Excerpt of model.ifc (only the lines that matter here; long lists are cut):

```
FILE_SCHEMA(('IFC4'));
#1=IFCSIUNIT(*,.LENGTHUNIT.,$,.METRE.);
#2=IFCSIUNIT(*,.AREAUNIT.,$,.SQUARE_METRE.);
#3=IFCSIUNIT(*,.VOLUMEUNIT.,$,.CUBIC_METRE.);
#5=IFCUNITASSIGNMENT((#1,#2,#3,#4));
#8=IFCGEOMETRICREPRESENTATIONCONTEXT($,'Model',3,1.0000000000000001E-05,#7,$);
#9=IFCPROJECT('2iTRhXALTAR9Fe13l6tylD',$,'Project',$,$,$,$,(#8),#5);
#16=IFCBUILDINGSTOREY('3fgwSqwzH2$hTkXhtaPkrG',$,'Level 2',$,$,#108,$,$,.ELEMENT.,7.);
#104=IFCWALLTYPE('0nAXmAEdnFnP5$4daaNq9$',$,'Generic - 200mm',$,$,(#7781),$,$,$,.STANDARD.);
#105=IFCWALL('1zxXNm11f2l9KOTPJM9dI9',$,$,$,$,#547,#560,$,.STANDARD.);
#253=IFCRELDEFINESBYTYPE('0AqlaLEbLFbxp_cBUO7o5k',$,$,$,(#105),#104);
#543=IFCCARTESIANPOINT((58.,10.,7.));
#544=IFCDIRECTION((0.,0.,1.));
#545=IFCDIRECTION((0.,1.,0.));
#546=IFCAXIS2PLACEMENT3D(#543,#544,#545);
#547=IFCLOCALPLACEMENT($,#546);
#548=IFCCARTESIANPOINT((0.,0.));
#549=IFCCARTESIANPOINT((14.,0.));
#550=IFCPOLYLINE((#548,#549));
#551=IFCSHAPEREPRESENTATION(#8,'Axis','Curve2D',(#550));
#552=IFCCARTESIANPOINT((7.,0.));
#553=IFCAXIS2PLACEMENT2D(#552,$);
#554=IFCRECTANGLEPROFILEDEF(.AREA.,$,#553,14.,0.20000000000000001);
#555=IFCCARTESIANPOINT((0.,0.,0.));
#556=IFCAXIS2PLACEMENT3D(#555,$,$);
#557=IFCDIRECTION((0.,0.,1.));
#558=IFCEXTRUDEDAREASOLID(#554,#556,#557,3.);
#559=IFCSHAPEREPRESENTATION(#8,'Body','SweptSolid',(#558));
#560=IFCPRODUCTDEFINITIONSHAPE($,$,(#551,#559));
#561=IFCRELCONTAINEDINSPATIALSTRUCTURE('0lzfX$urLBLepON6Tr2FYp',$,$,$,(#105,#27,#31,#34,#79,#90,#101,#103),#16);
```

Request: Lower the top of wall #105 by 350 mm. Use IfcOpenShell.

```python
import ifcopenshell
import ifcopenshell.geom
import ifcopenshell.util.shape
import ifcopenshell.util.unit

model = ifcopenshell.open("model.ifc")
unit_scale = ifcopenshell.util.unit.calculate_unit_scale(model)
settings = ifcopenshell.geom.settings()


def volume(element):
    """Net volume in cubic metres, openings subtracted."""
    shape = ifcopenshell.geom.create_shape(settings, element)
    return ifcopenshell.util.shape.get_volume(shape.geometry)


wall = model.by_guid("1zxXNm11f2l9KOTPJM9dI9")
before = volume(wall)

body = next(r for r in wall.Representation.Representations if r.RepresentationIdentifier == "Body")
solid = body.Items[0]
old_height = solid.Depth
solid.Depth -= 0.35 / unit_scale
after = volume(wall)

print(f"height {old_height:g} -> {solid.Depth:g}, volume {before:.3f} -> {after:.3f} m3")

model.write("model_rev.ifc")
```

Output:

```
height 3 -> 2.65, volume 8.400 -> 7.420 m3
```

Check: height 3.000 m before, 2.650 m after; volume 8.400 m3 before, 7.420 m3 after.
